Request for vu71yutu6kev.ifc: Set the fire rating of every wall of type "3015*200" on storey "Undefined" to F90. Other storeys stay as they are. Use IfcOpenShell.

First a look at what the model holds.

```python
import ifcopenshell
import ifcopenshell.util.element

model = ifcopenshell.open("vu71yutu6kev.ifc")
print(model.schema)
storey = next(s for s in model.by_type("IfcBuildingStorey") if s.Name == "Undefined")
walls = [e for e in ifcopenshell.util.element.get_decomposition(storey) if e.is_a("IfcWall")]
seen = {}
for e in walls:
    element_type = ifcopenshell.util.element.get_type(e)
    key = (element_type.Name if element_type != e and element_type else None, ifcopenshell.util.element.get_pset(e, "Pset_WallCommon", "FireRating"))
    seen[key] = seen.get(key, 0) + 1
for (name, value), count in sorted(seen.items(), key=str):
    print(count, "x", name, "|", value)
```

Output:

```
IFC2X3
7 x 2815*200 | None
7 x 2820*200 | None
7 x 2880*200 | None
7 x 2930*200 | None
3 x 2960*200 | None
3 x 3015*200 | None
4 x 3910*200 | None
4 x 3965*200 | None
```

```python
import ifcopenshell
import ifcopenshell.api.pset
import ifcopenshell.util.element

model = ifcopenshell.open("vu71yutu6kev.ifc")

storey = next(s for s in model.by_type("IfcBuildingStorey") if s.Name == "Undefined")
walls = [e for e in ifcopenshell.util.element.get_decomposition(storey) if e.is_a("IfcWall")]

count = 0
for e in walls:
    element_type = ifcopenshell.util.element.get_type(e)
    if element_type in (None, e) or element_type.Name != "3015*200":
        continue
    # add_pset returns the element's existing set when there is one.
    pset = ifcopenshell.api.pset.add_pset(model, product=e, name="Pset_WallCommon")
    ifcopenshell.api.pset.edit_pset(model, pset=pset, properties={"FireRating": "F90"})
    count += 1

print(count, "walls updated")

model.write("vu71yutu6kev_v2.ifc")
```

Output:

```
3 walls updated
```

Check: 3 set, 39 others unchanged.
